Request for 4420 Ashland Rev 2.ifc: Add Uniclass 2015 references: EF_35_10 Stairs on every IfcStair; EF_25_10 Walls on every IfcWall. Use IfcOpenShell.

First a look at what the model holds.

```python
import ifcopenshell

model = ifcopenshell.open("4420 Ashland Rev 2.ifc")
print(model.schema)
print("classifications:", [c.Name for c in model.by_type("IfcClassification")])
for ifc_class in ("IfcDoor", "IfcRoof", "IfcStair", "IfcWall", "IfcWindow"):
    print(ifc_class, len(model.by_type(ifc_class)))
```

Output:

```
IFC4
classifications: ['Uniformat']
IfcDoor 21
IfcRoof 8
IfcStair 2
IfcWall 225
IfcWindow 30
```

```python
import ifcopenshell
import ifcopenshell.api.classification

model = ifcopenshell.open("4420 Ashland Rev 2.ifc")

system = ifcopenshell.api.classification.add_classification(model, classification="Uniclass 2015")

codes = {
    "IfcStair": ("EF_35_10", "Stairs"),
    "IfcWall": ("EF_25_10", "Walls"),
}
for ifc_class, (code, name) in codes.items():
    products = model.by_type(ifc_class)
    ifcopenshell.api.classification.add_reference(
        model, products=products, classification=system, identification=code, name=name
    )
    print(code, len(products))

model.write("4420 Ashland Rev 2_rev.ifc")
```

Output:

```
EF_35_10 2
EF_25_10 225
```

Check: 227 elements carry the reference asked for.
